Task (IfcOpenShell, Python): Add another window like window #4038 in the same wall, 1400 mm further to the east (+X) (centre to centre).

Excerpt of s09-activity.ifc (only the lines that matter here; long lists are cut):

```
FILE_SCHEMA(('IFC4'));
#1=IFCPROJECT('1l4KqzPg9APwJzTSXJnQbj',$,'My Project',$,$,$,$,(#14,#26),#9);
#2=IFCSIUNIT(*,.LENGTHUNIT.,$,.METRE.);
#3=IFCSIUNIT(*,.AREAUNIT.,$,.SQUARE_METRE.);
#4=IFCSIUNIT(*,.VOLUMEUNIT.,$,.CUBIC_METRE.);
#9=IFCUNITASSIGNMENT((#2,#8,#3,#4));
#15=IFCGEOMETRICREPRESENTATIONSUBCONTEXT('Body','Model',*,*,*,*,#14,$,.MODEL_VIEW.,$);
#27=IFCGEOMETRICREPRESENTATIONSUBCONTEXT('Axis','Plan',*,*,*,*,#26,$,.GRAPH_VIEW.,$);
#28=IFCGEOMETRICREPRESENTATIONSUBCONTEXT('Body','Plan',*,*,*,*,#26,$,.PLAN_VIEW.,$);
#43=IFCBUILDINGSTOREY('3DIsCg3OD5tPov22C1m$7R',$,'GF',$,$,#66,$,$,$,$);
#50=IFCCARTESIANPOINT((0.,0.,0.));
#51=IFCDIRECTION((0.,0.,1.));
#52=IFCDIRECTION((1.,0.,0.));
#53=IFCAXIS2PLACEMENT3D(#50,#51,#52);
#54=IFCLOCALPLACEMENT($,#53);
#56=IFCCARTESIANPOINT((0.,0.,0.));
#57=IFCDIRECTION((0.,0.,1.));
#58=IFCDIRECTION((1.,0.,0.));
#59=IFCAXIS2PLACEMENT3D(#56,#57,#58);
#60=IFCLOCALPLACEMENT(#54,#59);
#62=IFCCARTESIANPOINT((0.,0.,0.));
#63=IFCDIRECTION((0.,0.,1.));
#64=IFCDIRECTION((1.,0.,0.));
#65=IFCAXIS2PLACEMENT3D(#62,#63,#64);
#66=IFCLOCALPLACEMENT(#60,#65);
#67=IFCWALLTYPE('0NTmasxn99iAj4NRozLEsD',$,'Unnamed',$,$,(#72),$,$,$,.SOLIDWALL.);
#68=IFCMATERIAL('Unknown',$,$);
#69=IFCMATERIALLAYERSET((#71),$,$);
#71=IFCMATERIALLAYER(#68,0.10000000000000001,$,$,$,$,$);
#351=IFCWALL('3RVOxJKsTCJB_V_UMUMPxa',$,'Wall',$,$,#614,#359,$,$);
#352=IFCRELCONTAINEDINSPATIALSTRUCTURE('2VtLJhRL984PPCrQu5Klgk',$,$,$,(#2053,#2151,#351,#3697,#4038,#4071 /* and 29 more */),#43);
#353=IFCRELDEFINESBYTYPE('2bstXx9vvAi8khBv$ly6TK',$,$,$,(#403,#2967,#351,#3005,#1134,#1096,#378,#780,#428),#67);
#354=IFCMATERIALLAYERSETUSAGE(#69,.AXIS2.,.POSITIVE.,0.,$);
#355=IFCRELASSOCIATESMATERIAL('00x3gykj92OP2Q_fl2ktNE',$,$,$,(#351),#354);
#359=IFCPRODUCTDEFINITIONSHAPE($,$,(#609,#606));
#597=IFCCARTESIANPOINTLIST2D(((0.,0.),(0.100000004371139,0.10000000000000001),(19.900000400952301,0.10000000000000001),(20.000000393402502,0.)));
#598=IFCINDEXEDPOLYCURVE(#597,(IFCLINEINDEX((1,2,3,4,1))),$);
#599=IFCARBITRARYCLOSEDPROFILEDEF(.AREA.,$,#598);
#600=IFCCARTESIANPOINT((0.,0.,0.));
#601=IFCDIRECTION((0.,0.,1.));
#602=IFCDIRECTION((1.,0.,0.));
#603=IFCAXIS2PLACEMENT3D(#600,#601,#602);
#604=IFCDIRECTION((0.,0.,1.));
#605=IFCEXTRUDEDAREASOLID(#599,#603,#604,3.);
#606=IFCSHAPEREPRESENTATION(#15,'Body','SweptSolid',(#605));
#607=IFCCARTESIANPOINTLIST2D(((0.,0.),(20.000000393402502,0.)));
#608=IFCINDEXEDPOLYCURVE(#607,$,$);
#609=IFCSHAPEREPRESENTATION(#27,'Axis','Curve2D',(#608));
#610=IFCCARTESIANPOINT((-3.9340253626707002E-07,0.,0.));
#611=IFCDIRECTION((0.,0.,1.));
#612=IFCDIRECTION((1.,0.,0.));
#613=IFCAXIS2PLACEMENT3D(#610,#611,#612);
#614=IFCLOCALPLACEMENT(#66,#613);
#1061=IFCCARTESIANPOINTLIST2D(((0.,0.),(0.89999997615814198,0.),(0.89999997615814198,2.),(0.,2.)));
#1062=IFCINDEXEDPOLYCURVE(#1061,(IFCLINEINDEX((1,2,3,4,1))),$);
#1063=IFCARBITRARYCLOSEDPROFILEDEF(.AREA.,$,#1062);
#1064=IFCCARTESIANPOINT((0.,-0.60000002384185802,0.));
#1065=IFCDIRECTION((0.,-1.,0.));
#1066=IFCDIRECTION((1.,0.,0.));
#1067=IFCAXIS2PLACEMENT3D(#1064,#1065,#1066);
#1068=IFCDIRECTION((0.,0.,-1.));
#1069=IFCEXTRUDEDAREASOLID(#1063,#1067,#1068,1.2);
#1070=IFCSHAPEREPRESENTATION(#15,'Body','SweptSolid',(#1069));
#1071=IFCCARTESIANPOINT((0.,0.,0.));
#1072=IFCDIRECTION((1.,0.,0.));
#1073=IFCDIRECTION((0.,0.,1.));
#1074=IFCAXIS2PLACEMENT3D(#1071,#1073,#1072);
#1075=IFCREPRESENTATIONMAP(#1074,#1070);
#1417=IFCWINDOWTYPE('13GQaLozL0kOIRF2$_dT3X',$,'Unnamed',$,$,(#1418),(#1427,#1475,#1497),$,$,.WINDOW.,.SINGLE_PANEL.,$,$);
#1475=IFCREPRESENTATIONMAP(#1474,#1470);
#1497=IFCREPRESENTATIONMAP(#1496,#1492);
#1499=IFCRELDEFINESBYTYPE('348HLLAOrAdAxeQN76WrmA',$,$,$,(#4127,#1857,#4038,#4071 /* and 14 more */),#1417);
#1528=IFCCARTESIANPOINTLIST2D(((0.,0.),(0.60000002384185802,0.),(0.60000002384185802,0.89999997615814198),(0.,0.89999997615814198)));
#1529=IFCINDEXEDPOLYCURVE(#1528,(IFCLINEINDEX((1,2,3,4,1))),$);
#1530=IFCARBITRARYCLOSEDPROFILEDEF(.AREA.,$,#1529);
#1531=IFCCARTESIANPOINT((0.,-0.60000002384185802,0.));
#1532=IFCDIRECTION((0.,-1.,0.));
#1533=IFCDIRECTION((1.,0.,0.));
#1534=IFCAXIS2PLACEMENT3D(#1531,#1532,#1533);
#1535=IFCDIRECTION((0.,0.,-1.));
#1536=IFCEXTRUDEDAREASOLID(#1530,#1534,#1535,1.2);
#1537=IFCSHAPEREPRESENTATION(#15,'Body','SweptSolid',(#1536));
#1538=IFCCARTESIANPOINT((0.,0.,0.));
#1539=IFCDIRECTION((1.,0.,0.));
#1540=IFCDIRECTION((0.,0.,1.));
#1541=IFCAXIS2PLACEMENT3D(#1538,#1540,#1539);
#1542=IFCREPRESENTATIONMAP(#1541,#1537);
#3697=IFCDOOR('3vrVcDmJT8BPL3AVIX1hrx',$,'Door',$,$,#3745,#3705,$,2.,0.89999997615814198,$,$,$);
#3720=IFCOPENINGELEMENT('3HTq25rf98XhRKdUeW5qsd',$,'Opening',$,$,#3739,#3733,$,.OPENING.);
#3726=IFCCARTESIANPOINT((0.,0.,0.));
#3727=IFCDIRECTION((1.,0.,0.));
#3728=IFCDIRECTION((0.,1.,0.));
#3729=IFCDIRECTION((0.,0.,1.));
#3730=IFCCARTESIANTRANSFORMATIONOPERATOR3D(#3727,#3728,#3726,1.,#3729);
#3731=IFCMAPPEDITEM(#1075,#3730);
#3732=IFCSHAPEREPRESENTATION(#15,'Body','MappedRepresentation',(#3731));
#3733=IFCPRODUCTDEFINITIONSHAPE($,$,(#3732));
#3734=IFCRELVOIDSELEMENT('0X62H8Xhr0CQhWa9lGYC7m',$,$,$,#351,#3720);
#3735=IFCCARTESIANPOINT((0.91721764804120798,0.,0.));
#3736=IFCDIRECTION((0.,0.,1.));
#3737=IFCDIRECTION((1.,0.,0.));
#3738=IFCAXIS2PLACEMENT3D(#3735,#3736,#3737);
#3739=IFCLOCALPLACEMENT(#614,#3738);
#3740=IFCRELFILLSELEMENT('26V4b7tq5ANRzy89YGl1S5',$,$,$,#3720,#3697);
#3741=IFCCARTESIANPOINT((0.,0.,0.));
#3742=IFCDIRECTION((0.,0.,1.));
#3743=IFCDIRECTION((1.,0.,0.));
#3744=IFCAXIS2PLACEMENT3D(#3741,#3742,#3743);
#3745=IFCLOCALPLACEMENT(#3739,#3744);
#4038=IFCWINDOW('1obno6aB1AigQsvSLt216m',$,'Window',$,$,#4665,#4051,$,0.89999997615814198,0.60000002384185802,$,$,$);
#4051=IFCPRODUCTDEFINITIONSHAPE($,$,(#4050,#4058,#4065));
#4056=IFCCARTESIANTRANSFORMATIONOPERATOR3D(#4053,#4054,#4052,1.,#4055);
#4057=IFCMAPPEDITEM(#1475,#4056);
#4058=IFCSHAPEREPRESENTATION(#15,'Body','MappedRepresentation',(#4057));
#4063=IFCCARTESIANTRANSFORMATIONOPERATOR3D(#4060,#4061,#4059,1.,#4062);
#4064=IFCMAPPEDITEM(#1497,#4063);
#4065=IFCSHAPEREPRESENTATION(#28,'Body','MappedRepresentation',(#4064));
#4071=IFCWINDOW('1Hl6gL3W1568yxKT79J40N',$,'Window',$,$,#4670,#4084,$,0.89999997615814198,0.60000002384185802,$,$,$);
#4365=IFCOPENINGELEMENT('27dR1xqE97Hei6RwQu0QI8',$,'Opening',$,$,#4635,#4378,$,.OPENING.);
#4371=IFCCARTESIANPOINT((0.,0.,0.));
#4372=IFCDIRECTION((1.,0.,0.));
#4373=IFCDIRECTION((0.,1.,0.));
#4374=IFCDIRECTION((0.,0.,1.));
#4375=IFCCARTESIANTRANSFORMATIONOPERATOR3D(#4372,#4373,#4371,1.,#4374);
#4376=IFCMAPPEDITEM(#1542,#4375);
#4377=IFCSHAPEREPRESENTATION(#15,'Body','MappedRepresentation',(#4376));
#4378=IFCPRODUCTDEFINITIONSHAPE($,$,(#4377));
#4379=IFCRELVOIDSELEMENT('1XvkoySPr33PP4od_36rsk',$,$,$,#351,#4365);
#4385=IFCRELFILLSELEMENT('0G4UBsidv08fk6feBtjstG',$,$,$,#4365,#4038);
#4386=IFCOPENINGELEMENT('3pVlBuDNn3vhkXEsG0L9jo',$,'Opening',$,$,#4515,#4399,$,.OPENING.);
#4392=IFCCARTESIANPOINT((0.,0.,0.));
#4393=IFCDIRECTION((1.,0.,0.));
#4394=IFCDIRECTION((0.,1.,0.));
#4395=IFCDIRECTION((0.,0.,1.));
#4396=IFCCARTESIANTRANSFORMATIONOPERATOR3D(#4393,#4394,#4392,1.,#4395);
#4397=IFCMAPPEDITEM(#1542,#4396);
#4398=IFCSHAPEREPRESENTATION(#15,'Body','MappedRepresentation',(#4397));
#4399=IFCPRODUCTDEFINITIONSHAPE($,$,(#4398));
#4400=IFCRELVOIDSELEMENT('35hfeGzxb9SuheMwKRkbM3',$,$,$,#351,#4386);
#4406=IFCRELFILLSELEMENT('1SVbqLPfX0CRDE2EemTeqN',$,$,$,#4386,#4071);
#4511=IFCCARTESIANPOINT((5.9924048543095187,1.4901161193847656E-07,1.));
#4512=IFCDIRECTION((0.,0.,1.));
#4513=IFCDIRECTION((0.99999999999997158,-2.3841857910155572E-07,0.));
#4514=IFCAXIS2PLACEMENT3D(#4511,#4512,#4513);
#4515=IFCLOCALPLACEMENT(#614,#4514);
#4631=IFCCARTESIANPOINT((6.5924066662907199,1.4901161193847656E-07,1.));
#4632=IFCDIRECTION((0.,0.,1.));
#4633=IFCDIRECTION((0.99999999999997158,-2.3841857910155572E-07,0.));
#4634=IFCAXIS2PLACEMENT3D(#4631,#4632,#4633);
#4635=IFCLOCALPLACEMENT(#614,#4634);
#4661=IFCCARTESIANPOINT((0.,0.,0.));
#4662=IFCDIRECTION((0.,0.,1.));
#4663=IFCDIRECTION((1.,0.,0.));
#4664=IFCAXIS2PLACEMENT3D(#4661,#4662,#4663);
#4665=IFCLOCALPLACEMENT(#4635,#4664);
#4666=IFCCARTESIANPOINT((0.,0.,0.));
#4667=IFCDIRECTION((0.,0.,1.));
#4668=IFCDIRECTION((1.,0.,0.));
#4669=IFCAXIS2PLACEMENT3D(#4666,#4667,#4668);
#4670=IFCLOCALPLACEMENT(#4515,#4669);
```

```python
import ifcopenshell
import ifcopenshell.api.feature
import ifcopenshell.api.geometry
import ifcopenshell.api.root
import ifcopenshell.geom
import ifcopenshell.util.element
import ifcopenshell.util.placement
import ifcopenshell.util.shape
import ifcopenshell.util.unit

model = ifcopenshell.open("s09-activity.ifc")
unit_scale = ifcopenshell.util.unit.calculate_unit_scale(model)
settings = ifcopenshell.geom.settings()


def volume(element):
    """Net volume in cubic metres, openings subtracted."""
    shape = ifcopenshell.geom.create_shape(settings, element)
    return ifcopenshell.util.shape.get_volume(shape.geometry)


window = model.by_guid("1obno6aB1AigQsvSLt216m")
opening = window.FillsVoids[0].RelatingOpeningElement
wall = opening.VoidsElements[0].RelatingBuildingElement
before = volume(wall)
shift = ifcopenshell.util.placement.get_local_placement(wall.ObjectPlacement)[:3, 0] * 1.4 / unit_scale

# copy_class copies the void relationship, type, container and properties, but no geometry.
new_opening = ifcopenshell.api.root.copy_class(model, product=opening)
new_opening.Representation = ifcopenshell.util.element.copy_deep(
    model, opening.Representation, exclude=["IfcGeometricRepresentationContext", "IfcRepresentationMap"]
)
new_window = ifcopenshell.api.root.copy_class(model, product=window)
new_window.Representation = ifcopenshell.util.element.copy_deep(
    model, window.Representation, exclude=["IfcGeometricRepresentationContext", "IfcRepresentationMap"]
)
ifcopenshell.api.feature.add_filling(model, opening=new_opening, element=new_window)

for old, new in ((opening, new_opening), (window, new_window)):
    matrix = ifcopenshell.util.placement.get_local_placement(old.ObjectPlacement)
    matrix[:3, 3] += shift
    ifcopenshell.api.geometry.edit_object_placement(model, product=new, matrix=matrix, is_si=False)

after = volume(wall)

print(f"wall volume {before:.3f} -> {after:.3f} m3")

model.write("s09-activity_updated.ifc")
```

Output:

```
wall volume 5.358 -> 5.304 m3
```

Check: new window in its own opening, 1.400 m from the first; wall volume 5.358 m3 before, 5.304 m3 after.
